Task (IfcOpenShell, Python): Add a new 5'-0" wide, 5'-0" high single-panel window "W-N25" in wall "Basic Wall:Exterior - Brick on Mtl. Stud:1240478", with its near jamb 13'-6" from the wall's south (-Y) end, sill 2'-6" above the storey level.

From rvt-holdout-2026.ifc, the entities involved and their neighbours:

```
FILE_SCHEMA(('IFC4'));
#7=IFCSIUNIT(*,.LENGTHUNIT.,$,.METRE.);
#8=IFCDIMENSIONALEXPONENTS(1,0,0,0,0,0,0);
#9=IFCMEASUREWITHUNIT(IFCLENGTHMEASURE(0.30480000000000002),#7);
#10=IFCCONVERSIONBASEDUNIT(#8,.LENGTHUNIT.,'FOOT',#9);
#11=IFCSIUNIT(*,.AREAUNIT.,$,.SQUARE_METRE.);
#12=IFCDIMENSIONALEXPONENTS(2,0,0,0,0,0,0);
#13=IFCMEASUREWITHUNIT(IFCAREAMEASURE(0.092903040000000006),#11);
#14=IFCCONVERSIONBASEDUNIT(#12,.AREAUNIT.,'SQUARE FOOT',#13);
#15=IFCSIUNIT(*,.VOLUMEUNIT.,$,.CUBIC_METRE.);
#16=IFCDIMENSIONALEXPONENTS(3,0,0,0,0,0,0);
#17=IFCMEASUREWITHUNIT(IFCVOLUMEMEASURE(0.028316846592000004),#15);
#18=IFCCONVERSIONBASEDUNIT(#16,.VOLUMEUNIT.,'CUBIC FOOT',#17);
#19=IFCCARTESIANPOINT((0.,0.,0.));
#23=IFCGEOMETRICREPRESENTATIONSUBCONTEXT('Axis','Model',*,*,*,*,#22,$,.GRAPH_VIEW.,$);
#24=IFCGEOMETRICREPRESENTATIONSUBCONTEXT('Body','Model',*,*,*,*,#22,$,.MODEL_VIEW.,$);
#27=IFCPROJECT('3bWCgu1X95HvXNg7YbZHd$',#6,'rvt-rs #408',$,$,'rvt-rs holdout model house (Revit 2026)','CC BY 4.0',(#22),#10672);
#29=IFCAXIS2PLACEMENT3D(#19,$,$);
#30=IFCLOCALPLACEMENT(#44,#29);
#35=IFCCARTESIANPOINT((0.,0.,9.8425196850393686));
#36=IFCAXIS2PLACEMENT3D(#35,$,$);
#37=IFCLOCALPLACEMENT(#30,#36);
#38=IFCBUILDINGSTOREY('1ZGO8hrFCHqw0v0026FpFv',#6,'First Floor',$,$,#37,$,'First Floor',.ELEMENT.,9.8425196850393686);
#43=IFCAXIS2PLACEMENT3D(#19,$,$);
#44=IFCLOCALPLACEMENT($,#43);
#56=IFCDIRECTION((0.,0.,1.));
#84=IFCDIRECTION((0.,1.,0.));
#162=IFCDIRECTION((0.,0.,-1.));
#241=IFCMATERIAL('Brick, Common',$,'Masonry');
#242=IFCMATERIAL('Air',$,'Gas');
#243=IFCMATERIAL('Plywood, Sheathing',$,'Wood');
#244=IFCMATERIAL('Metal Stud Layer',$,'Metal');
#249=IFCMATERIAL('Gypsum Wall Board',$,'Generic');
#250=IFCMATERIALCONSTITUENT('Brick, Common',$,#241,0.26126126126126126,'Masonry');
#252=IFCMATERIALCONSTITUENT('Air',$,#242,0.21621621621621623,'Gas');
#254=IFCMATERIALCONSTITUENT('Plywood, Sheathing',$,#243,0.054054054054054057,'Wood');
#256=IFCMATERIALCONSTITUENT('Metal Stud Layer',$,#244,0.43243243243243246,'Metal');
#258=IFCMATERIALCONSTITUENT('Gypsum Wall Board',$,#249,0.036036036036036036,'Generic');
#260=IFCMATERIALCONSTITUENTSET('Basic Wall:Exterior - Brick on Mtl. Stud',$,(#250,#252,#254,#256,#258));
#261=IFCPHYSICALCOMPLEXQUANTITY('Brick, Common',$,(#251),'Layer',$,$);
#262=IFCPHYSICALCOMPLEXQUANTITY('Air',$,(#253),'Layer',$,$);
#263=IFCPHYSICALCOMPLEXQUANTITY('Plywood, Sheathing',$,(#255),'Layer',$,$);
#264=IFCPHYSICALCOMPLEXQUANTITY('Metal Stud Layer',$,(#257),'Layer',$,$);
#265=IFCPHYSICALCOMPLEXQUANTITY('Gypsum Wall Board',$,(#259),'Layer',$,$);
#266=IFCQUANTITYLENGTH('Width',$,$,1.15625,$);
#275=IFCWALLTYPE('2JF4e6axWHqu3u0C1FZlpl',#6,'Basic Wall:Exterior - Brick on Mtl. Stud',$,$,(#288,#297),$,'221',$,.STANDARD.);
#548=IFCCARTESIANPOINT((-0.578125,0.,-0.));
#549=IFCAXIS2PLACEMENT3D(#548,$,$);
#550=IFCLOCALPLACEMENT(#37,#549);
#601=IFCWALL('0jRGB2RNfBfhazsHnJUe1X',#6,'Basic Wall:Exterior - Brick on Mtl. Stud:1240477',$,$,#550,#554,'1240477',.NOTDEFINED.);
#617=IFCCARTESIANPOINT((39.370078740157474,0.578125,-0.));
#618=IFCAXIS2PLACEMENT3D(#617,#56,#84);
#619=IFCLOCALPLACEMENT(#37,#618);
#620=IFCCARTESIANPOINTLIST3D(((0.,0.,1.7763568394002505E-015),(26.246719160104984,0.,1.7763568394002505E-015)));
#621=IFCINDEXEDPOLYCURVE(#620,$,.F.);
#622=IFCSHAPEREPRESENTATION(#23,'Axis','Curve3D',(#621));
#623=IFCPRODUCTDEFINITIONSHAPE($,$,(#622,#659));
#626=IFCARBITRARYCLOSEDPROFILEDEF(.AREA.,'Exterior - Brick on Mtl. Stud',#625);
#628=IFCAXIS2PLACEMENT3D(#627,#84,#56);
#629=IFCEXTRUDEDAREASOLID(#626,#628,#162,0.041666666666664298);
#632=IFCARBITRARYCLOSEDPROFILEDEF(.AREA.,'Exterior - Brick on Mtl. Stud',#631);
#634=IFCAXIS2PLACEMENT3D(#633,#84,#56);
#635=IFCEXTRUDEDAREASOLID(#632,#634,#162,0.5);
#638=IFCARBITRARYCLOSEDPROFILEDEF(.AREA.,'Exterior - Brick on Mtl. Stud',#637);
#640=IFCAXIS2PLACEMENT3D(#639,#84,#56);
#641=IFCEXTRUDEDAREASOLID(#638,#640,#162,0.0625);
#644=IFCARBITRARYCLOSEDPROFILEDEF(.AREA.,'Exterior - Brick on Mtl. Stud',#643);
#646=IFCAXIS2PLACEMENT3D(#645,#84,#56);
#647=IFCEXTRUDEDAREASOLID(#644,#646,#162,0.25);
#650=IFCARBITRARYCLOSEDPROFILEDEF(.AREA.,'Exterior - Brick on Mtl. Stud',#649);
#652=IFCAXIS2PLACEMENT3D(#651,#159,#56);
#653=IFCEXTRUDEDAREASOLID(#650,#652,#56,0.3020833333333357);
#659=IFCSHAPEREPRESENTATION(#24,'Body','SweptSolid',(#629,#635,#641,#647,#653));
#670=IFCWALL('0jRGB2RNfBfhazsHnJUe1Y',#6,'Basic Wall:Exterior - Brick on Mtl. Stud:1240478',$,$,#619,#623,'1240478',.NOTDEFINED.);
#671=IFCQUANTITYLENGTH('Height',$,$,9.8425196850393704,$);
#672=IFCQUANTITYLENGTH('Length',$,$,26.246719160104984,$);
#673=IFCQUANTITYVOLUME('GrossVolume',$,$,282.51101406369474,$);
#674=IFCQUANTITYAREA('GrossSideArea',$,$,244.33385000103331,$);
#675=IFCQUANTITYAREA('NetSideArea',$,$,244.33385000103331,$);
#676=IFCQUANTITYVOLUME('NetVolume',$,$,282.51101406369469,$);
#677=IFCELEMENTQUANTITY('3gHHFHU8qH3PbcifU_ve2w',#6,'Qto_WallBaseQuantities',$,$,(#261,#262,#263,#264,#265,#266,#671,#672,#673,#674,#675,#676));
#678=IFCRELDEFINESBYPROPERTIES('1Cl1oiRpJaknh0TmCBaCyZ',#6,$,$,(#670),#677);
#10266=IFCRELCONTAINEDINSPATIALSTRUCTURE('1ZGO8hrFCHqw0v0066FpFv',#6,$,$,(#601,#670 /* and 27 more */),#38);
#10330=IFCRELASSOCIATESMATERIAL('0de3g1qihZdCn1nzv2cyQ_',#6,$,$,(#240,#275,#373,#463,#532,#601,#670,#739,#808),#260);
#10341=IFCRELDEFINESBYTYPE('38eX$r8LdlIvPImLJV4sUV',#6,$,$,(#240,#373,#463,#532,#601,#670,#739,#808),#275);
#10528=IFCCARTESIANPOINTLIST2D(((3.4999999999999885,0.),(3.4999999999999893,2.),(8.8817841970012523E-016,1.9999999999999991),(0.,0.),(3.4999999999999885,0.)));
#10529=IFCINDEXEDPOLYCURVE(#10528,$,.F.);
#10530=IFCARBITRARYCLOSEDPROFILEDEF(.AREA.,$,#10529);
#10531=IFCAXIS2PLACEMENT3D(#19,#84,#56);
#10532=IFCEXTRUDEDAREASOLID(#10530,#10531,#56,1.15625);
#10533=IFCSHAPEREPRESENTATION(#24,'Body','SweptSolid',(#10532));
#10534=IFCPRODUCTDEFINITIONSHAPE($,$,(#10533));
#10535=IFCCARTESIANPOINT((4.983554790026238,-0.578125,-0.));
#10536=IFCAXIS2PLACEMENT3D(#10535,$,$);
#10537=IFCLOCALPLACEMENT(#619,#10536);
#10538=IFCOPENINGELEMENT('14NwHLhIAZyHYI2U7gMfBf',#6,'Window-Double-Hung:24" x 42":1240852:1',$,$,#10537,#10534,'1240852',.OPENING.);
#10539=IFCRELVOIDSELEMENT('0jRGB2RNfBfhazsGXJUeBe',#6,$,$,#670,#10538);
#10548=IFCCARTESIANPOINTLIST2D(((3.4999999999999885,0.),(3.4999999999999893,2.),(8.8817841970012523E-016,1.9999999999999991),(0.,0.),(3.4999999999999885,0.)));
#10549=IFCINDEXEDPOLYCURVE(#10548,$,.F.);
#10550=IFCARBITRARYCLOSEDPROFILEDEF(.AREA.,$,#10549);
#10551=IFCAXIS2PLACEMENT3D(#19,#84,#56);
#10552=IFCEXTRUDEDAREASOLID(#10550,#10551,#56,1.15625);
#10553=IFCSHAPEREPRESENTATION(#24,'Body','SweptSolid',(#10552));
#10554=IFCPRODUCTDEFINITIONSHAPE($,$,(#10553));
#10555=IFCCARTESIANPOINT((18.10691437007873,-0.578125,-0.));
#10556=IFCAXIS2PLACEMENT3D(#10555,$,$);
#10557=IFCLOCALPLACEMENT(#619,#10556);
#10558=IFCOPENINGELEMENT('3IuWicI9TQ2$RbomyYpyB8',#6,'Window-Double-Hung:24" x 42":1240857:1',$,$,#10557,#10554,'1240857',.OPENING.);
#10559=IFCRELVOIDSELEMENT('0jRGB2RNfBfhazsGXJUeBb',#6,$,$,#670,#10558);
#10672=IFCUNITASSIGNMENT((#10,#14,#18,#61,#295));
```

```python
import numpy as np
import ifcopenshell
import ifcopenshell.api.feature
import ifcopenshell.api.geometry
import ifcopenshell.api.pset
import ifcopenshell.api.root
import ifcopenshell.api.spatial
import ifcopenshell.geom
import ifcopenshell.util.element
import ifcopenshell.util.placement
import ifcopenshell.util.representation
import ifcopenshell.util.shape
import ifcopenshell.util.unit

model = ifcopenshell.open("rvt-holdout-2026.ifc")
unit_scale = ifcopenshell.util.unit.calculate_unit_scale(model)
area_scale = ifcopenshell.util.unit.calculate_unit_scale(model, "AREAUNIT")
volume_scale = ifcopenshell.util.unit.calculate_unit_scale(model, "VOLUMEUNIT")
settings = ifcopenshell.geom.settings()


def volume(element):
    """Net volume in cubic metres, openings subtracted."""
    shape = ifcopenshell.geom.create_shape(settings, element)
    return ifcopenshell.util.shape.get_volume(shape.geometry)


wall = model.by_id(670)
storey = ifcopenshell.util.element.get_container(wall, ifc_class="IfcBuildingStorey")
context = ifcopenshell.util.representation.get_context(model, "Model", "Body", "MODEL_VIEW")
before = volume(wall)

width, height, from_end, sill = 1.524, 1.524, 4.1148, 0.762  # metres

# The wall runs along its own X axis, and the end named is its -X end.
wall_shape = ifcopenshell.geom.create_shape(settings, wall)
x, y, z = ifcopenshell.util.shape.get_vertices(wall_shape.geometry).T
start = x.min() + from_end
face, thickness = float(y.min()), float(y.max() - y.min())
wall_matrix = ifcopenshell.util.placement.get_local_placement(wall.ObjectPlacement)
level = ifcopenshell.util.placement.get_local_placement(storey.ObjectPlacement)[2, 3]


def in_wall(x, y):
    """Placement at x, y metres in the wall's axes, at sill height."""
    matrix = wall_matrix.copy()
    matrix[:, 3] = wall_matrix @ np.array([x / unit_scale, y / unit_scale, 0.0, 1.0])
    matrix[2, 3] = level + sill / unit_scale
    return matrix


# Opening: a box that overshoots both wall faces by 50 mm.
opening = ifcopenshell.api.root.create_entity(model, ifc_class="IfcOpeningElement", predefined_type="OPENING")
box = ifcopenshell.api.geometry.add_wall_representation(
    model, context=context, length=width, height=height, thickness=thickness + 0.1
)
ifcopenshell.api.geometry.assign_representation(model, product=opening, representation=box)
ifcopenshell.api.geometry.edit_object_placement(model, product=opening, matrix=in_wall(start, face - 0.05), is_si=False)
ifcopenshell.api.feature.add_feature(model, feature=opening, element=wall)

window = ifcopenshell.api.root.create_entity(model, ifc_class="IfcWindow", name="W-N25", predefined_type="WINDOW")
window.OverallWidth, window.OverallHeight = width / unit_scale, height / unit_scale
window.PartitioningType = "SINGLE_PANEL"
body = ifcopenshell.api.geometry.add_window_representation(
    model,
    context=context,
    overall_width=window.OverallWidth,
    overall_height=window.OverallHeight,
    partition_type="SINGLE_PANEL",
)
ifcopenshell.api.geometry.assign_representation(model, product=window, representation=body)
ifcopenshell.api.spatial.assign_container(model, products=[window], relating_structure=storey)
ifcopenshell.api.feature.add_filling(model, opening=opening, element=window)

# Centre the window in the wall's thickness.
ifcopenshell.api.geometry.edit_object_placement(model, product=window, matrix=in_wall(start, face), is_si=False)
window_shape = ifcopenshell.geom.create_shape(settings, window)
depth = ifcopenshell.util.shape.get_vertices(window_shape.geometry)[:, 1]
offset = face + thickness / 2 - (depth.min() + depth.max()) / 2
ifcopenshell.api.geometry.edit_object_placement(model, product=window, matrix=in_wall(start, offset), is_si=False)

after = volume(wall)

# Update the wall's stored quantities.
qto = model.by_id(ifcopenshell.util.element.get_pset(wall, "Qto_WallBaseQuantities", should_inherit=False)["id"])
ifcopenshell.api.pset.edit_qto(model, qto=qto, properties={
    "NetSideArea": after / thickness / area_scale,
    "NetVolume": after / volume_scale,
})

print(f"wall volume {before:.3f} -> {after:.3f} m3")

model.write("rvt-holdout-2026_edited.ifc")
```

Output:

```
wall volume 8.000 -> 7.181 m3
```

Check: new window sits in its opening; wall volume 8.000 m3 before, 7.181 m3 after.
